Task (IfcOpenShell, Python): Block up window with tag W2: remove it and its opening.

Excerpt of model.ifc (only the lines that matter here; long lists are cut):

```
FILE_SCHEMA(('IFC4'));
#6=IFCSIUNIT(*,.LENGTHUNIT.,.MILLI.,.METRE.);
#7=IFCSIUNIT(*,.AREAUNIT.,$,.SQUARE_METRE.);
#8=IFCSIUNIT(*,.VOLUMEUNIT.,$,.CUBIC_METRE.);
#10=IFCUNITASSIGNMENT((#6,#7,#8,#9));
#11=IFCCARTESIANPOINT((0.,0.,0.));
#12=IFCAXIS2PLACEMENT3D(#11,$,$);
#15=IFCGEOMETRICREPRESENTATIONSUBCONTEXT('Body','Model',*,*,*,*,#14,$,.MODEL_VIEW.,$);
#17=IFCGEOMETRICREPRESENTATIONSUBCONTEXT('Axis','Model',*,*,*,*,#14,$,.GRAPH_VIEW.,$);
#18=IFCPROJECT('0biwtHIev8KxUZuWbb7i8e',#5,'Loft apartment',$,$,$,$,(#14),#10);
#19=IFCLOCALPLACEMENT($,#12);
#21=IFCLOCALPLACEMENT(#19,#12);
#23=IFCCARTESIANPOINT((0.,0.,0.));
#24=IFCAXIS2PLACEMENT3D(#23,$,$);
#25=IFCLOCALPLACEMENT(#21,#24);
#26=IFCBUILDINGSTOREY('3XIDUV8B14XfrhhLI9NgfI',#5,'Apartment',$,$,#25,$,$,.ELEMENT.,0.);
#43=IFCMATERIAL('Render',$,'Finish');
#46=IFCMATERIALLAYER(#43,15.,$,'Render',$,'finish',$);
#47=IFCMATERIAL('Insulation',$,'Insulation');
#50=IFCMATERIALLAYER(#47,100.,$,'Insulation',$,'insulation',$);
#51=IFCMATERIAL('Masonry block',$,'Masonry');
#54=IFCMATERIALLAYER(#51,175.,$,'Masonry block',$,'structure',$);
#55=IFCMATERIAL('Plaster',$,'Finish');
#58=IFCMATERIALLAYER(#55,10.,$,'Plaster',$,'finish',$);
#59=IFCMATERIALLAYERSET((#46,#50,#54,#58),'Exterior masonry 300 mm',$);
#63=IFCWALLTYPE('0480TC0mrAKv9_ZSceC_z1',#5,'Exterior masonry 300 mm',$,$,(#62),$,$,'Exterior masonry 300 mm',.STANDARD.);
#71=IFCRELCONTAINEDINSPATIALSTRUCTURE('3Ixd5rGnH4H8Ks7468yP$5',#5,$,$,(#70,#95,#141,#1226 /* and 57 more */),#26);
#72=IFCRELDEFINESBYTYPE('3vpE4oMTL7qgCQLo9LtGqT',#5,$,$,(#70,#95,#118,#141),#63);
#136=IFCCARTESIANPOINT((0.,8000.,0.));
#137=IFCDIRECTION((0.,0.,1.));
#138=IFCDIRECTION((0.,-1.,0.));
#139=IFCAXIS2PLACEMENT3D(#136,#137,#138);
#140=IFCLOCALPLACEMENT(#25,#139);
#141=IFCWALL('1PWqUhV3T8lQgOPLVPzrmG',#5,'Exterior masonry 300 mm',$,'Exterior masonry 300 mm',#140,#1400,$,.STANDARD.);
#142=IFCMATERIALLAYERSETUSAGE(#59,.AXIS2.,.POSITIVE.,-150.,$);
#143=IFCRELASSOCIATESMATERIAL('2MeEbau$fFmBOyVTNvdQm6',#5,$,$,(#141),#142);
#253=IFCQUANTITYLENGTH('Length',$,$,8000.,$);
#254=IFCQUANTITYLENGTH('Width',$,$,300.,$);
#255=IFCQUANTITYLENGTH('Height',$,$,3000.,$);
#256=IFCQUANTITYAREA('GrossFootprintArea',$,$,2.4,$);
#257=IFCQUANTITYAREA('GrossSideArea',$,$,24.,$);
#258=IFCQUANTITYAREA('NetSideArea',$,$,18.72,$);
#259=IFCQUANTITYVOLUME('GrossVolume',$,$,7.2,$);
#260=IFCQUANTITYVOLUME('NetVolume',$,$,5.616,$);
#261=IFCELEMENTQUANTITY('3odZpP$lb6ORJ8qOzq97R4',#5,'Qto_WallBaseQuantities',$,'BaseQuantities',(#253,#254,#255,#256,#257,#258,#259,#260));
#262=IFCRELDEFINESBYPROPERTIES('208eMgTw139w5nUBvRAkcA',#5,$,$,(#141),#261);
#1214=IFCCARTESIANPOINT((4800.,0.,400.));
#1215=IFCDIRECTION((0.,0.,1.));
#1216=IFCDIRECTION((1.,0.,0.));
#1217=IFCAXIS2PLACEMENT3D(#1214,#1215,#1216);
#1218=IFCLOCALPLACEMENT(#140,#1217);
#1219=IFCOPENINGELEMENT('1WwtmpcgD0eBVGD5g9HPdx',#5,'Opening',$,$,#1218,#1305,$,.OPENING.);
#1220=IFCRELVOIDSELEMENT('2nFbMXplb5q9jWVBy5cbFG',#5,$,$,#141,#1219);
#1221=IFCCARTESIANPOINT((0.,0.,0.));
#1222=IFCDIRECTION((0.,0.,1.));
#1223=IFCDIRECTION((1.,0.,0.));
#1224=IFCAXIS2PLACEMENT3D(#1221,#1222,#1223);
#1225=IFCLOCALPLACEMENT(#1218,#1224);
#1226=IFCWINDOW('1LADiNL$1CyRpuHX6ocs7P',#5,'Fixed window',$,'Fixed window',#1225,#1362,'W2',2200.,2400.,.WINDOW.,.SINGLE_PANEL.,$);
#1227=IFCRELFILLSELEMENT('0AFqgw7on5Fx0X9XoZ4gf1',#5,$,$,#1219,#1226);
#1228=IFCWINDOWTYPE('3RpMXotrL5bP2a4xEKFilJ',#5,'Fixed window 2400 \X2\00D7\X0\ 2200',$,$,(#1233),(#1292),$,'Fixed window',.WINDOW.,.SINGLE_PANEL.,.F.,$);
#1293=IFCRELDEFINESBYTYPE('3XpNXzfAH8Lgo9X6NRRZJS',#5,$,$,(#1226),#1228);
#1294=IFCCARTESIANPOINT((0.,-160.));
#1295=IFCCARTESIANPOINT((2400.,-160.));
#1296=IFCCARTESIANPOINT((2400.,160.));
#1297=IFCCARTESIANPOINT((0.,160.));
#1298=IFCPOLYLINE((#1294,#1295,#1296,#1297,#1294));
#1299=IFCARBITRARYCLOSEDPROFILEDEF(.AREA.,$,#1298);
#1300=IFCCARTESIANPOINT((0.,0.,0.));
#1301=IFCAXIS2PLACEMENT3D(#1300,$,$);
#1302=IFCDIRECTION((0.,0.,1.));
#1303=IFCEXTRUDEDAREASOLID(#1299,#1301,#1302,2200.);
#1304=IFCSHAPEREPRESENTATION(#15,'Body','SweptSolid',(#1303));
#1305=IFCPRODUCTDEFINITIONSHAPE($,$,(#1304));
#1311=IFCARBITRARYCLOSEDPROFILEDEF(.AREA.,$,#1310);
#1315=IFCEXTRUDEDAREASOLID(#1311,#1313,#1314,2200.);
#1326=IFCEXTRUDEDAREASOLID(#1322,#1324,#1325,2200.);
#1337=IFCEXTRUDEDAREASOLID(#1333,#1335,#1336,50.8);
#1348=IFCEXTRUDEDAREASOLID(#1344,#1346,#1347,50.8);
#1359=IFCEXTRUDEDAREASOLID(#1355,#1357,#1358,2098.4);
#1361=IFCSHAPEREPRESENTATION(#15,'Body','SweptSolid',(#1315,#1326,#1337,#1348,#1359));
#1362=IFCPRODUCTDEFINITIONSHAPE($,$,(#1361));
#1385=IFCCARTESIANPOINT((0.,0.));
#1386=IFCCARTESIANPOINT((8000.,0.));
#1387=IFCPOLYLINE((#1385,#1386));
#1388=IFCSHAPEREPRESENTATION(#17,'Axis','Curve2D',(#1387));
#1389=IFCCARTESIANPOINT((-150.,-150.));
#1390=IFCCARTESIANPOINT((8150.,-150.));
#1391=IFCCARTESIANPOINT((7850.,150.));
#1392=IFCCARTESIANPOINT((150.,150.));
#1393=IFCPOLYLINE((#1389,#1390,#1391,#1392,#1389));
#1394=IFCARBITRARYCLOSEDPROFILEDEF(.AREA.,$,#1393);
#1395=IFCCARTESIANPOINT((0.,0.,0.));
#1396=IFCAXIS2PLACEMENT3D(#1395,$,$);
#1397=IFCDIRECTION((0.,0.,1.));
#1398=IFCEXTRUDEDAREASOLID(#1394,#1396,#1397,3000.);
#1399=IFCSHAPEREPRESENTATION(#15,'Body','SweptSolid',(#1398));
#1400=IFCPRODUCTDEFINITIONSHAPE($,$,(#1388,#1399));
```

```python
import ifcopenshell
import ifcopenshell.api.feature
import ifcopenshell.api.pset
import ifcopenshell.api.root
import ifcopenshell.geom
import ifcopenshell.util.element
import ifcopenshell.util.shape
import ifcopenshell.util.unit

model = ifcopenshell.open("model.ifc")
area_scale = ifcopenshell.util.unit.calculate_unit_scale(model, "AREAUNIT")
volume_scale = ifcopenshell.util.unit.calculate_unit_scale(model, "VOLUMEUNIT")
settings = ifcopenshell.geom.settings()


def volume(element):
    """Net volume in cubic metres, openings subtracted."""
    shape = ifcopenshell.geom.create_shape(settings, element)
    return ifcopenshell.util.shape.get_volume(shape.geometry)


window = model.by_guid("1LADiNL$1CyRpuHX6ocs7P")
opening = window.FillsVoids[0].RelatingOpeningElement
wall = opening.VoidsElements[0].RelatingBuildingElement
before = volume(wall)

ifcopenshell.api.root.remove_product(model, product=window)
ifcopenshell.api.feature.remove_feature(model, feature=opening)

after = volume(wall)
thickness = 0.3  # wall thickness in metres

# Update the wall's stored quantities.
qto = model.by_id(ifcopenshell.util.element.get_pset(wall, "Qto_WallBaseQuantities", should_inherit=False)["id"])
ifcopenshell.api.pset.edit_qto(model, qto=qto, properties={
    "NetSideArea": after / thickness / area_scale,
    "NetVolume": after / volume_scale,
})

print(f"wall volume {before:.3f} -> {after:.3f} m3")

model.write("model-out.ifc")
```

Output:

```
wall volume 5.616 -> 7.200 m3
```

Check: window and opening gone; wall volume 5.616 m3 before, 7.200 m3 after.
